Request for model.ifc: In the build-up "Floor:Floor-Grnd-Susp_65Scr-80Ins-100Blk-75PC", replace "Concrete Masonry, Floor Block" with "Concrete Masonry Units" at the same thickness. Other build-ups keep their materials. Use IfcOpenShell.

First a look at what the model holds.

```python
import ifcopenshell
import ifcopenshell.util.element

model = ifcopenshell.open("model.ifc")
print(model.schema)
for layer_set in model.by_type("IfcMaterialLayerSet"):
    if layer_set.LayerSetName == "Floor:Floor-Grnd-Susp_65Scr-80Ins-100Blk-75PC":
        for layer in layer_set.MaterialLayers:
            print(layer.id(), layer.Material and layer.Material.Name, layer.LayerThickness, sep=" | ")
        print(len(ifcopenshell.util.element.get_elements_by_material(model, layer_set)), "elements and types use it")
print(sorted(m.Name for m in model.by_type("IfcMaterial") if m.Name)[:60])
```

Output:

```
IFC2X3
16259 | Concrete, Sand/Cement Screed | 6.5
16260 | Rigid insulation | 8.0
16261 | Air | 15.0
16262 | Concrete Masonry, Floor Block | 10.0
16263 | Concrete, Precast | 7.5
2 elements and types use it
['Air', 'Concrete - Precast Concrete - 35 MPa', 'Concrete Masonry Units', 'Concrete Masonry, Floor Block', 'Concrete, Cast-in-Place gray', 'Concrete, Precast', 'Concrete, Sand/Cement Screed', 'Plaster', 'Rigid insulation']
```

```python
import ifcopenshell
import ifcopenshell.api.material

model = ifcopenshell.open("model.ifc")

layer_set = next(s for s in model.by_type("IfcMaterialLayerSet") if s.LayerSetName == "Floor:Floor-Grnd-Susp_65Scr-80Ins-100Blk-75PC")
layer = next(l for l in layer_set.MaterialLayers if l.Material and l.Material.Name == "Concrete Masonry, Floor Block")
material = next(m for m in model.by_type("IfcMaterial") if m.Name == "Concrete Masonry Units")

# Point this one layer at the other material; renaming the old one would change it everywhere.
ifcopenshell.api.material.edit_layer(model, layer=layer, attributes={}, material=material)

print([l.Material.Name if l.Material else None for l in layer_set.MaterialLayers])

model.write("model_v2.ifc")
```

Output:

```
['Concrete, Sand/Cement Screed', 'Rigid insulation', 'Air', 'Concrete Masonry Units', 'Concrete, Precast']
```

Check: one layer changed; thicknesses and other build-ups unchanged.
